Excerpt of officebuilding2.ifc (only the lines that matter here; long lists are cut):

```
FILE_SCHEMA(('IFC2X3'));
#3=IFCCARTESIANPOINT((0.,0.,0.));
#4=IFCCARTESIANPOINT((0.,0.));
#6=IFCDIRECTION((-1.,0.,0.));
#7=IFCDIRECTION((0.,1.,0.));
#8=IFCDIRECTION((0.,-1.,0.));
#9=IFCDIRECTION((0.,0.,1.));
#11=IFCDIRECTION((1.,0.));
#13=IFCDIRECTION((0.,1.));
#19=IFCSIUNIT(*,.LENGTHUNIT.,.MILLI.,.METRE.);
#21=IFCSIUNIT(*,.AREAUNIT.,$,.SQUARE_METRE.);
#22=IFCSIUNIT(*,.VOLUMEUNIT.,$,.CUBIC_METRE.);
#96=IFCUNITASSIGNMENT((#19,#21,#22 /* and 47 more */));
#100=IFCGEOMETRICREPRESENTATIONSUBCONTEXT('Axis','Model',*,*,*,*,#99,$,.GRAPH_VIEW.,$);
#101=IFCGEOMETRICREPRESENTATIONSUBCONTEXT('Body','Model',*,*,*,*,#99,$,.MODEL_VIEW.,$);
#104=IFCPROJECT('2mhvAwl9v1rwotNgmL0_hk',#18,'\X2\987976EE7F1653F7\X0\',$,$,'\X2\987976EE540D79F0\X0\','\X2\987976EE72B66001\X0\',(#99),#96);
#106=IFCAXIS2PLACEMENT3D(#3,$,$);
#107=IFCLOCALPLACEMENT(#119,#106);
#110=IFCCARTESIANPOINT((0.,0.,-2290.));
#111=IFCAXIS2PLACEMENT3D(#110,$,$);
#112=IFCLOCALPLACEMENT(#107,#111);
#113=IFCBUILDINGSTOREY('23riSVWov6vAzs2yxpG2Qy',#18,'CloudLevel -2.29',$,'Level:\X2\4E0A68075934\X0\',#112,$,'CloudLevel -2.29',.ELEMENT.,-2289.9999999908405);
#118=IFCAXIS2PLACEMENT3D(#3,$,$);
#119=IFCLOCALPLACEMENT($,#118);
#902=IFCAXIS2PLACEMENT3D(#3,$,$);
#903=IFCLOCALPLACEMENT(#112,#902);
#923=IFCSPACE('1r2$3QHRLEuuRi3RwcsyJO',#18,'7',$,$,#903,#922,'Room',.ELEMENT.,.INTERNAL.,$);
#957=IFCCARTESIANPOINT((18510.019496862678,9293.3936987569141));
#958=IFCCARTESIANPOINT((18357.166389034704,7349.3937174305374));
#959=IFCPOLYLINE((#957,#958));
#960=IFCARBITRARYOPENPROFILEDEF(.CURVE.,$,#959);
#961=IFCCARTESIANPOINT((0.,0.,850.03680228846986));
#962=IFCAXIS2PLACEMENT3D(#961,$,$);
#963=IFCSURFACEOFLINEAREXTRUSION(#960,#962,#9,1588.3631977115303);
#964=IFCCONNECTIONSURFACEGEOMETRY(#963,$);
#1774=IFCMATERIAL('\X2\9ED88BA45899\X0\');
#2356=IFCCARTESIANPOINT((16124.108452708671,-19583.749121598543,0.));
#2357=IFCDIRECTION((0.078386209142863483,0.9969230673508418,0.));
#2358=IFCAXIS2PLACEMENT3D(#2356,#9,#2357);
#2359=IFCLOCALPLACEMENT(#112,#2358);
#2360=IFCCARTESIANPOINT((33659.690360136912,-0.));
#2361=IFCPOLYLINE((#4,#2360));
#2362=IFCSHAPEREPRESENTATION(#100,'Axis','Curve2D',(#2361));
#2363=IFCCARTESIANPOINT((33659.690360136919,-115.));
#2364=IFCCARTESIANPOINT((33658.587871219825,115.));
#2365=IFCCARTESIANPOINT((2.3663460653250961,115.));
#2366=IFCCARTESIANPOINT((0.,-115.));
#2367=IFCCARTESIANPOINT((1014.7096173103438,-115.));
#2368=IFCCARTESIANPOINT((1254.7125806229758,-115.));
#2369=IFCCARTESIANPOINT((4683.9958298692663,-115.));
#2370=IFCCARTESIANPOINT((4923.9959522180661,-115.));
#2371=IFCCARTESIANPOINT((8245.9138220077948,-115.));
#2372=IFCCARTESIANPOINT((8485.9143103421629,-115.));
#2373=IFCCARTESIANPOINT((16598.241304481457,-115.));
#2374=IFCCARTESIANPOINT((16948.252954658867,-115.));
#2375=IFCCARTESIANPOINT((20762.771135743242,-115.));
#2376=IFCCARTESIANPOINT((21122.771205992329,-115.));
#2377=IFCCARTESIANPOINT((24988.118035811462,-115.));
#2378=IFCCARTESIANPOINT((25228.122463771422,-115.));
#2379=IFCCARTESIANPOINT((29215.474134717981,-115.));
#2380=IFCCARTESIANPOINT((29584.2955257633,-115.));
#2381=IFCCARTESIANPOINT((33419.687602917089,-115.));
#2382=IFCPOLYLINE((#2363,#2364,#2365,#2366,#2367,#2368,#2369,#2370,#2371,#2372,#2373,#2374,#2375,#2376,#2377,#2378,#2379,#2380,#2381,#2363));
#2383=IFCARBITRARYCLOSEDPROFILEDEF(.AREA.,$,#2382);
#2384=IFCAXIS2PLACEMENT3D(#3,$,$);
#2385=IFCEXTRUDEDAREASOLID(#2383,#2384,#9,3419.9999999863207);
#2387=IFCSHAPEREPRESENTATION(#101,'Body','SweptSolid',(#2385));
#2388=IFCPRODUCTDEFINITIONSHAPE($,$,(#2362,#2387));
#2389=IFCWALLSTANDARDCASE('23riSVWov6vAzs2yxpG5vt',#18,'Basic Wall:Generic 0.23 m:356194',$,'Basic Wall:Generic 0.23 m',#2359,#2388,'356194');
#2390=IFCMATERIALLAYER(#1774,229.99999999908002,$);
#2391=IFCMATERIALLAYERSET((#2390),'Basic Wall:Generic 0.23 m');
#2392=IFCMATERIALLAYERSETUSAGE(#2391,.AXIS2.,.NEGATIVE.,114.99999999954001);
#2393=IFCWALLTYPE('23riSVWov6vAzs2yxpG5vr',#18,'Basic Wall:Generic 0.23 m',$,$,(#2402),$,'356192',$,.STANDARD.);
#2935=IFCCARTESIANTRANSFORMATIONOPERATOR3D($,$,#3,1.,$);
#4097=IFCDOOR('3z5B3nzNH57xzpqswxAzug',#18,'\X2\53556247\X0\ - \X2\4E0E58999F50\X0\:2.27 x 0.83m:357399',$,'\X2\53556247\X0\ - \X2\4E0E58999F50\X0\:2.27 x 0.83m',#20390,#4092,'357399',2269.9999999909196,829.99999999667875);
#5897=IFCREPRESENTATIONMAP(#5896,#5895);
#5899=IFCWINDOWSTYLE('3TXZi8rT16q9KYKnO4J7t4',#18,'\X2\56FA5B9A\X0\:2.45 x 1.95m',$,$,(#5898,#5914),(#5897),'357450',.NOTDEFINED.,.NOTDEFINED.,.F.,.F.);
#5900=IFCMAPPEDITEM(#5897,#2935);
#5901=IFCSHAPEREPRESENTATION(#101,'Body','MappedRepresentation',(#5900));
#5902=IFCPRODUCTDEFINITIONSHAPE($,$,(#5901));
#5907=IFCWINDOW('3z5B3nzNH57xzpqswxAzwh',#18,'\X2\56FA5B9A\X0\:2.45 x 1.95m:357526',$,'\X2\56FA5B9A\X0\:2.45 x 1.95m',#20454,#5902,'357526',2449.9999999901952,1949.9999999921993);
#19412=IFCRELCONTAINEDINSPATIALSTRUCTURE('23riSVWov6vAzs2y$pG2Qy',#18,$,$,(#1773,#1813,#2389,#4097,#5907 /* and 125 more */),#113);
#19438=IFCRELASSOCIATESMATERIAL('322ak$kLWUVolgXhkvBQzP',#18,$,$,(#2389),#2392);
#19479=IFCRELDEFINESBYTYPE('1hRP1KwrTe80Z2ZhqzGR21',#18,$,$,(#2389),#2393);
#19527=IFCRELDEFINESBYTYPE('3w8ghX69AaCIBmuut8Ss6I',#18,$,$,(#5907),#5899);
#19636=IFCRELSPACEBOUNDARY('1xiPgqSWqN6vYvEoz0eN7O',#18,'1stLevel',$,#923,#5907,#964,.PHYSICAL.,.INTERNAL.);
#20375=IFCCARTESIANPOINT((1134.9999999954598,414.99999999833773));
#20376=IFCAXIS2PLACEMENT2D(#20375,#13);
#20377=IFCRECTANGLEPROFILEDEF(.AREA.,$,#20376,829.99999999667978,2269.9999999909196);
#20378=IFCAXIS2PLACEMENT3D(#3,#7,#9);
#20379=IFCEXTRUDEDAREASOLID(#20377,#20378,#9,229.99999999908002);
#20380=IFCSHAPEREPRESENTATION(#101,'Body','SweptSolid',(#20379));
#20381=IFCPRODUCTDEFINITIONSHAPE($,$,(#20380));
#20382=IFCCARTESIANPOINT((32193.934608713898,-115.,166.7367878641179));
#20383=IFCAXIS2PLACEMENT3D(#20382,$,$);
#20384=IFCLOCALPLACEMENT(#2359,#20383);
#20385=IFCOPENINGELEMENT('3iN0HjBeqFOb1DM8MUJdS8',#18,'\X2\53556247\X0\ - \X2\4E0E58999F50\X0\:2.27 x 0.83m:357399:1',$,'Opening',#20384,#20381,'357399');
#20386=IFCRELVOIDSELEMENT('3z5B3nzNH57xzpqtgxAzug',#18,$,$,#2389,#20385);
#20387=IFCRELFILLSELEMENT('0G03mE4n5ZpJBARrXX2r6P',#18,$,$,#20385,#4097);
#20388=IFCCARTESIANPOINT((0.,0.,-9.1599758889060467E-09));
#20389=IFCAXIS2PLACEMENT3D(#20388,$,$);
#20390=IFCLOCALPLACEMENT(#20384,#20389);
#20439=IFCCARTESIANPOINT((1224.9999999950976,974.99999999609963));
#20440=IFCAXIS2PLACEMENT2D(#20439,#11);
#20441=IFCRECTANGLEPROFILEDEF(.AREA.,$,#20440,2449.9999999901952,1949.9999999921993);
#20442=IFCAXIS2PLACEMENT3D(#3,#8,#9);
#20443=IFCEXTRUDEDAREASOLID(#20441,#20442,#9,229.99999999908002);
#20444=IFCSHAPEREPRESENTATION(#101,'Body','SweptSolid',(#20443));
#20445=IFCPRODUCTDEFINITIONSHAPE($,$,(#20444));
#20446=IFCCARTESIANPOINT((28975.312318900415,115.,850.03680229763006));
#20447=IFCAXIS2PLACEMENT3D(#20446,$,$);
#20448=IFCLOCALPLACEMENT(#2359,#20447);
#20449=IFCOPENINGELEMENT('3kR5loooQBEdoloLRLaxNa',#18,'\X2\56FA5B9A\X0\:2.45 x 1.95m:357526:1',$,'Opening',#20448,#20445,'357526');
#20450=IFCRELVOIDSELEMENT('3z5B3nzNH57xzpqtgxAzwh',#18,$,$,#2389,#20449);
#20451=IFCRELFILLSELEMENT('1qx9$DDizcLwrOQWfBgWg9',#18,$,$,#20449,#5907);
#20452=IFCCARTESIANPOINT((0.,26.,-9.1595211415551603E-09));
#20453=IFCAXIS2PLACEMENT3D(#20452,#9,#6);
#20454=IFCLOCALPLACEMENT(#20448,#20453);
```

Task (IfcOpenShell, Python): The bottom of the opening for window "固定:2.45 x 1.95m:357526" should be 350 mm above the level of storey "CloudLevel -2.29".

```python
import numpy as np
import ifcopenshell
import ifcopenshell.api.geometry
import ifcopenshell.geom
import ifcopenshell.util.element
import ifcopenshell.util.placement
import ifcopenshell.util.shape
import ifcopenshell.util.unit

model = ifcopenshell.open("officebuilding2.ifc")
unit_scale = ifcopenshell.util.unit.calculate_unit_scale(model)

window = model.by_id(5907)
opening = window.FillsVoids[0].RelatingOpeningElement
storey = ifcopenshell.util.element.get_container(window, ifc_class="IfcBuildingStorey")
level = ifcopenshell.util.placement.get_local_placement(storey.ObjectPlacement)[2, 3]

# The opening's origin need not be at the sill, so measure its lowest point.
shape = ifcopenshell.geom.create_shape(ifcopenshell.geom.settings(), opening)
bottom = ifcopenshell.util.shape.get_shape_bottom_elevation(shape, shape.geometry) / unit_scale
dz = level + 0.35 / unit_scale - bottom

shift = np.array([0.0, 0.0, dz])
# The window is placed relative to its opening, so it follows when the opening moves.
matrix = ifcopenshell.util.placement.get_local_placement(opening.ObjectPlacement)
matrix[:3, 3] += shift
ifcopenshell.api.geometry.edit_object_placement(
    model, product=opening, matrix=matrix, is_si=False, should_transform_children=True
)

# Space boundary surfaces are stored in each space's coordinates; move them too.
for rel in window.ProvidesBoundaries:
    if not rel.ConnectionGeometry:
        continue
    surface = rel.ConnectionGeometry.SurfaceOnRelatingElement
    space_matrix = ifcopenshell.util.placement.get_local_placement(rel.RelatingSpace.ObjectPlacement)
    point = np.array(surface.Position.Location.Coordinates) + space_matrix[:3, :3].T @ shift
    surface.Position = model.createIfcAxis2Placement3D(
        model.createIfcCartesianPoint(point.tolist()), surface.Position.Axis, surface.Position.RefDirection
    )

print(f"moved by {dz * unit_scale:+.3f} m")

model.write("officebuilding2_v2.ifc")
```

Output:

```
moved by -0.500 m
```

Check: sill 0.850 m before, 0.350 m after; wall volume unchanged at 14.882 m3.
